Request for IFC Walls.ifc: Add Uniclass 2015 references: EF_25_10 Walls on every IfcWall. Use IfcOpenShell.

First a look at what the model holds.

```python
import ifcopenshell

model = ifcopenshell.open("IFC Walls.ifc")
print(model.schema)
print("classifications:", [c.Name for c in model.by_type("IfcClassification")])
for ifc_class in ("IfcDoor", "IfcRoof", "IfcStair", "IfcWall", "IfcWindow"):
    print(ifc_class, len(model.by_type(ifc_class)))
```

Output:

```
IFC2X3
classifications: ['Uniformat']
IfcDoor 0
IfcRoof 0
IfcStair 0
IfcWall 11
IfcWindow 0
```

```python
import ifcopenshell
import ifcopenshell.api.classification

model = ifcopenshell.open("IFC Walls.ifc")

# IFC2X3 requires Source and Edition and has no link from the project to the system.
system = model.create_entity("IfcClassification", Source="NBS", Edition="2015", Name="Uniclass 2015")

codes = {
    "IfcWall": ("EF_25_10", "Walls"),
}
for ifc_class, (code, name) in codes.items():
    products = model.by_type(ifc_class)
    ifcopenshell.api.classification.add_reference(
        model, products=products, classification=system, identification=code, name=name
    )
    print(code, len(products))

model.write("IFC Walls-out.ifc")
```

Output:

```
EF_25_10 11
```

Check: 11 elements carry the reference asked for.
